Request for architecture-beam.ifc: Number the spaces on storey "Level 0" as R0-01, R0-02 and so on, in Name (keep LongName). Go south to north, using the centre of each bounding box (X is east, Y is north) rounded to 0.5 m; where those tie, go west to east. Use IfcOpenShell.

First a look at what the model holds.

```python
import ifcopenshell
import ifcopenshell.util.element
import ifcopenshell.util.placement

model = ifcopenshell.open("architecture-beam.ifc")
print(model.schema)
storey = next(s for s in model.by_type("IfcBuildingStorey") if s.Name == "Level 0")
spaces = [e for e in ifcopenshell.util.element.get_decomposition(storey) if e.is_a("IfcSpace")]
for e in sorted(spaces, key=lambda e: e.id()):
    origin = ifcopenshell.util.placement.get_local_placement(e.ObjectPlacement)[:3, 3]
    print(e.id(), e.Name, e.LongName, origin.round(2) + 0.0, sep=" | ")
```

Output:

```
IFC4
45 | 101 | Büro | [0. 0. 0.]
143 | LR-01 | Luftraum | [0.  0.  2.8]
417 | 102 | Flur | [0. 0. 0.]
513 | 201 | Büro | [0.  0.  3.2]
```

```python
import ifcopenshell
import ifcopenshell.geom
import ifcopenshell.util.element
import ifcopenshell.util.shape

model = ifcopenshell.open("architecture-beam.ifc")
settings = ifcopenshell.geom.settings()
settings.set("use-world-coords", True)


def centre(element):
    shape = ifcopenshell.geom.create_shape(settings, element)
    return ifcopenshell.util.shape.get_bbox_centroid(shape.geometry)


storey = next(s for s in model.by_type("IfcBuildingStorey") if s.Name == "Level 0")
spaces = [e for e in ifcopenshell.util.element.get_decomposition(storey) if e.is_a("IfcSpace")]

# Insertion points can sit at a corner or the storey origin, so sort by the geometry (in metres).
centres = {e: centre(e) for e in spaces}
spaces.sort(key=lambda e: (round(centres[e][1] / 0.5), centres[e][0]))

for i, e in enumerate(spaces, start=1):
    number = f"R0-{i:02d}"
    e.Name = number
    print(e.id(), number)

model.write("architecture-beam_v2.ifc")
```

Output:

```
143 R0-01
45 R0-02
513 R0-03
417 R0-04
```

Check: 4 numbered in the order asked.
